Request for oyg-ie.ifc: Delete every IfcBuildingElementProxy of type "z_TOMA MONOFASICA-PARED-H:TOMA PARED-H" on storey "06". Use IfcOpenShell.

First a look at what the model holds.

```python
import ifcopenshell
import ifcopenshell.util.element

model = ifcopenshell.open("oyg-ie.ifc")
print(model.schema)
storey = next(s for s in model.by_type("IfcBuildingStorey") if s.Name == "06")
proxies = [e for e in ifcopenshell.util.element.get_decomposition(storey) if e.is_a("IfcBuildingElementProxy")]
seen = {}
for e in proxies:
    element_type = ifcopenshell.util.element.get_type(e)
    name = element_type.Name if element_type not in (None, e) else None
    seen[name] = seen.get(name, 0) + 1
for name, count in sorted(seen.items(), key=str):
    print(count, "x", name)
```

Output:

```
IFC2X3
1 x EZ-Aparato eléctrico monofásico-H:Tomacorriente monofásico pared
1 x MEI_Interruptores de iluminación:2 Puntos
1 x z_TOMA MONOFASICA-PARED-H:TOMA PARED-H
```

```python
import ifcopenshell
import ifcopenshell.api.root
import ifcopenshell.util.element

model = ifcopenshell.open("oyg-ie.ifc")

storey = next(s for s in model.by_type("IfcBuildingStorey") if s.Name == "06")
proxies = [e for e in ifcopenshell.util.element.get_decomposition(storey) if e.is_a("IfcBuildingElementProxy")]
targets = [e for e in proxies if (t := ifcopenshell.util.element.get_type(e)) not in (None, e) and t.Name == "z_TOMA MONOFASICA-PARED-H:TOMA PARED-H"]

for e in targets:
    ifcopenshell.api.root.remove_product(model, product=e)
print(len(targets), "removed")

model.write("oyg-ie_rev.ifc")
```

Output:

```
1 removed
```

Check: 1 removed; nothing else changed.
